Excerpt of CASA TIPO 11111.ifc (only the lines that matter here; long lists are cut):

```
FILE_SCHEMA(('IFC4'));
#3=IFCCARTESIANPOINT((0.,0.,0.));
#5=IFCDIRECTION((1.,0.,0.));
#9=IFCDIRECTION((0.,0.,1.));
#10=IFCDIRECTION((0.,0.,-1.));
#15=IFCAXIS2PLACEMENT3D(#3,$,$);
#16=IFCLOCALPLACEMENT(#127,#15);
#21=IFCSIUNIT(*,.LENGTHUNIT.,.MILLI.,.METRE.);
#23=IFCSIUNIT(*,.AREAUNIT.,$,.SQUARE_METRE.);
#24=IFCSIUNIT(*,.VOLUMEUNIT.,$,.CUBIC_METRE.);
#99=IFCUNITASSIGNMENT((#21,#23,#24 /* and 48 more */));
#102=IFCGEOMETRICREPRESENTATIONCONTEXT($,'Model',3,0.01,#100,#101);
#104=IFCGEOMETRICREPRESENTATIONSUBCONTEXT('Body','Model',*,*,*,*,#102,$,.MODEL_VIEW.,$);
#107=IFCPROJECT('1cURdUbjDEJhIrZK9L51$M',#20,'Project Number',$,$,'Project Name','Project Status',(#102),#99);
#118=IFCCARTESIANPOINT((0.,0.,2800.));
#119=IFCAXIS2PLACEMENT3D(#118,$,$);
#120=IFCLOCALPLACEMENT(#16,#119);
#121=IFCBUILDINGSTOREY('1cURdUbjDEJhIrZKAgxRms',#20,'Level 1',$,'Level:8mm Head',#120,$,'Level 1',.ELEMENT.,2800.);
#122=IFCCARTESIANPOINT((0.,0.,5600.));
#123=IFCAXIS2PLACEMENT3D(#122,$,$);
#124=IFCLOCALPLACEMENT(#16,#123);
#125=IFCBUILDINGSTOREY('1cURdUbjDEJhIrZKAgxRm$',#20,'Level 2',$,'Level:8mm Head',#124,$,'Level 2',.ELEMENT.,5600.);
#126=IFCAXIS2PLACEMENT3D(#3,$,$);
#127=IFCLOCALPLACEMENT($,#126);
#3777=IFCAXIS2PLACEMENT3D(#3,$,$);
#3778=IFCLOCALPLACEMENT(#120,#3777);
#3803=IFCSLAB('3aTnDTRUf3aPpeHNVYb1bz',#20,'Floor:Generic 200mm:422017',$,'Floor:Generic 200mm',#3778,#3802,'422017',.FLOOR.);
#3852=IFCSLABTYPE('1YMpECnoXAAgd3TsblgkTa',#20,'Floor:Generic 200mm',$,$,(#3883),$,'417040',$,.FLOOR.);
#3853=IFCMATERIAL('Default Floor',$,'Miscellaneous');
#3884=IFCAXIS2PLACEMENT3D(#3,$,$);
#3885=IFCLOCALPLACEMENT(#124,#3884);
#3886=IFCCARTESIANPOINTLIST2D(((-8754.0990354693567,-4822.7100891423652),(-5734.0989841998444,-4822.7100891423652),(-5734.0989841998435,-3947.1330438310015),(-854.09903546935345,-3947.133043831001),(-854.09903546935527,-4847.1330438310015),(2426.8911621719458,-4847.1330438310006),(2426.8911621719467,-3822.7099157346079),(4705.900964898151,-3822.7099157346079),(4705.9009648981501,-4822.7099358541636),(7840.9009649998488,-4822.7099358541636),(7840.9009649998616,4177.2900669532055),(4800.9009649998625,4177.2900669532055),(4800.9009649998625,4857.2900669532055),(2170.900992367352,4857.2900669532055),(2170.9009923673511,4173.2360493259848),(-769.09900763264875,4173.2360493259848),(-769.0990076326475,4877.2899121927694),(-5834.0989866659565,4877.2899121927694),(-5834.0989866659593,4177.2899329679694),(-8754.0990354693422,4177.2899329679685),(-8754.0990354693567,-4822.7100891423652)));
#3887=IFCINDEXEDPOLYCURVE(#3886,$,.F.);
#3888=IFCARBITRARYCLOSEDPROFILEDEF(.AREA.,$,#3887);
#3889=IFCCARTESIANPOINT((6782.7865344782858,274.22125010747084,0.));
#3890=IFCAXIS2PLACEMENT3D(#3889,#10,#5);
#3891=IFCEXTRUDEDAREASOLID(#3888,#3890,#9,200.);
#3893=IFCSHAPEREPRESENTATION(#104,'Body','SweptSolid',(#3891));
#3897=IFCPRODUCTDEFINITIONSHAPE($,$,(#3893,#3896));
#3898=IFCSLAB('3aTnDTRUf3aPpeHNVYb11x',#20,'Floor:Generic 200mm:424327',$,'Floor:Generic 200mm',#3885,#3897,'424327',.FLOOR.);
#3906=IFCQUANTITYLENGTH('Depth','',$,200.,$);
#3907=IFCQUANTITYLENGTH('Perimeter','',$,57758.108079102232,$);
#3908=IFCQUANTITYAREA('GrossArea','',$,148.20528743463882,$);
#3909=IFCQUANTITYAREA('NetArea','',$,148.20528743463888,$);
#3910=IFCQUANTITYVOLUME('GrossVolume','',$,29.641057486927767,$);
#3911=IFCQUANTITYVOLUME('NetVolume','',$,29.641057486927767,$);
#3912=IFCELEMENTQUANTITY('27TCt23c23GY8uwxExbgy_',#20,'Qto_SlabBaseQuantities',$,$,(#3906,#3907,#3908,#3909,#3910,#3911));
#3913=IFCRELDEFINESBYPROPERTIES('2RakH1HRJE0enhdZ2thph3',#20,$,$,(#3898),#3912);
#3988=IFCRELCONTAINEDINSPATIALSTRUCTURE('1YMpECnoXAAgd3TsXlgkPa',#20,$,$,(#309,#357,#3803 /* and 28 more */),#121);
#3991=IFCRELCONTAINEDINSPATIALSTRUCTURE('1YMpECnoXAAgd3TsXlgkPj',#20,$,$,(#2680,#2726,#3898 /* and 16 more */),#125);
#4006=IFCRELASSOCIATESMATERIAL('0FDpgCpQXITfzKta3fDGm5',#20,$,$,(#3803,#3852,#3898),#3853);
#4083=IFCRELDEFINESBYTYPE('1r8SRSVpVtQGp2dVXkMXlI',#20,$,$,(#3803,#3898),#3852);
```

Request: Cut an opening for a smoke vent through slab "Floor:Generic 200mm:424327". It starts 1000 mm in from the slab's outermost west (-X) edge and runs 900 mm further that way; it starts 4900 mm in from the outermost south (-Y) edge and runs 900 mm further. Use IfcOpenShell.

```python
import numpy as np
import ifcopenshell
import ifcopenshell.api.feature
import ifcopenshell.api.geometry
import ifcopenshell.api.pset
import ifcopenshell.api.root
import ifcopenshell.geom
import ifcopenshell.util.element
import ifcopenshell.util.placement
import ifcopenshell.util.representation
import ifcopenshell.util.shape
import ifcopenshell.util.unit

model = ifcopenshell.open("CASA TIPO 11111.ifc")
unit_scale = ifcopenshell.util.unit.calculate_unit_scale(model)
area_scale = ifcopenshell.util.unit.calculate_unit_scale(model, "AREAUNIT")
volume_scale = ifcopenshell.util.unit.calculate_unit_scale(model, "VOLUMEUNIT")
settings = ifcopenshell.geom.settings()


def volume(element):
    """Net volume in cubic metres, openings subtracted."""
    shape = ifcopenshell.geom.create_shape(settings, element)
    return ifcopenshell.util.shape.get_volume(shape.geometry)


slab = model.by_guid("3aTnDTRUf3aPpeHNVYb11x")
before = volume(slab)

# Extent in the slab's own axes, in metres. The edges named are its -X and -Y sides.
slab_shape = ifcopenshell.geom.create_shape(settings, slab)
vertices = ifcopenshell.util.shape.get_vertices(slab_shape.geometry)
x_min, y_min, bottom = vertices.min(axis=0)
top = vertices[:, 2].max()

opening = ifcopenshell.api.root.create_entity(model, ifc_class="IfcOpeningElement", name="Smoke vent opening", predefined_type="OPENING")
context = ifcopenshell.util.representation.get_context(model, "Model", "Body", "MODEL_VIEW")
width, depth = 0.9, 0.9
outline = [(0.0, 0.0), (width, 0.0), (width, depth), (0.0, depth), (0.0, 0.0)]
# Overshoot both faces by 50 mm so the cut is clean.
shape = ifcopenshell.api.geometry.add_slab_representation(
    model, context=context, depth=top - bottom + 0.1, polyline=outline
)
ifcopenshell.api.geometry.assign_representation(model, product=opening, representation=shape)

matrix = ifcopenshell.util.placement.get_local_placement(slab.ObjectPlacement)
matrix[:, 3] = matrix @ np.append(np.array([x_min + 1, y_min + 4.9, bottom - 0.05]) / unit_scale, 1.0)
ifcopenshell.api.geometry.edit_object_placement(model, product=opening, matrix=matrix, is_si=False)
ifcopenshell.api.feature.add_feature(model, feature=opening, element=slab)

after = volume(slab)

# Update the slab's stored quantities.
qto = model.by_id(ifcopenshell.util.element.get_pset(slab, "Qto_SlabBaseQuantities", should_inherit=False)["id"])
ifcopenshell.api.pset.edit_qto(model, qto=qto, properties={
    "NetArea": after / (top - bottom) / area_scale,
    "NetVolume": after / volume_scale,
})

print(f"slab volume {before:.3f} -> {after:.3f} m3")

model.write("CASA TIPO 11111_rev.ifc")
```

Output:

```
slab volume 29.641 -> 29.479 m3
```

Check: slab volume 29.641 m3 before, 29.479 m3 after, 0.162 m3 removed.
